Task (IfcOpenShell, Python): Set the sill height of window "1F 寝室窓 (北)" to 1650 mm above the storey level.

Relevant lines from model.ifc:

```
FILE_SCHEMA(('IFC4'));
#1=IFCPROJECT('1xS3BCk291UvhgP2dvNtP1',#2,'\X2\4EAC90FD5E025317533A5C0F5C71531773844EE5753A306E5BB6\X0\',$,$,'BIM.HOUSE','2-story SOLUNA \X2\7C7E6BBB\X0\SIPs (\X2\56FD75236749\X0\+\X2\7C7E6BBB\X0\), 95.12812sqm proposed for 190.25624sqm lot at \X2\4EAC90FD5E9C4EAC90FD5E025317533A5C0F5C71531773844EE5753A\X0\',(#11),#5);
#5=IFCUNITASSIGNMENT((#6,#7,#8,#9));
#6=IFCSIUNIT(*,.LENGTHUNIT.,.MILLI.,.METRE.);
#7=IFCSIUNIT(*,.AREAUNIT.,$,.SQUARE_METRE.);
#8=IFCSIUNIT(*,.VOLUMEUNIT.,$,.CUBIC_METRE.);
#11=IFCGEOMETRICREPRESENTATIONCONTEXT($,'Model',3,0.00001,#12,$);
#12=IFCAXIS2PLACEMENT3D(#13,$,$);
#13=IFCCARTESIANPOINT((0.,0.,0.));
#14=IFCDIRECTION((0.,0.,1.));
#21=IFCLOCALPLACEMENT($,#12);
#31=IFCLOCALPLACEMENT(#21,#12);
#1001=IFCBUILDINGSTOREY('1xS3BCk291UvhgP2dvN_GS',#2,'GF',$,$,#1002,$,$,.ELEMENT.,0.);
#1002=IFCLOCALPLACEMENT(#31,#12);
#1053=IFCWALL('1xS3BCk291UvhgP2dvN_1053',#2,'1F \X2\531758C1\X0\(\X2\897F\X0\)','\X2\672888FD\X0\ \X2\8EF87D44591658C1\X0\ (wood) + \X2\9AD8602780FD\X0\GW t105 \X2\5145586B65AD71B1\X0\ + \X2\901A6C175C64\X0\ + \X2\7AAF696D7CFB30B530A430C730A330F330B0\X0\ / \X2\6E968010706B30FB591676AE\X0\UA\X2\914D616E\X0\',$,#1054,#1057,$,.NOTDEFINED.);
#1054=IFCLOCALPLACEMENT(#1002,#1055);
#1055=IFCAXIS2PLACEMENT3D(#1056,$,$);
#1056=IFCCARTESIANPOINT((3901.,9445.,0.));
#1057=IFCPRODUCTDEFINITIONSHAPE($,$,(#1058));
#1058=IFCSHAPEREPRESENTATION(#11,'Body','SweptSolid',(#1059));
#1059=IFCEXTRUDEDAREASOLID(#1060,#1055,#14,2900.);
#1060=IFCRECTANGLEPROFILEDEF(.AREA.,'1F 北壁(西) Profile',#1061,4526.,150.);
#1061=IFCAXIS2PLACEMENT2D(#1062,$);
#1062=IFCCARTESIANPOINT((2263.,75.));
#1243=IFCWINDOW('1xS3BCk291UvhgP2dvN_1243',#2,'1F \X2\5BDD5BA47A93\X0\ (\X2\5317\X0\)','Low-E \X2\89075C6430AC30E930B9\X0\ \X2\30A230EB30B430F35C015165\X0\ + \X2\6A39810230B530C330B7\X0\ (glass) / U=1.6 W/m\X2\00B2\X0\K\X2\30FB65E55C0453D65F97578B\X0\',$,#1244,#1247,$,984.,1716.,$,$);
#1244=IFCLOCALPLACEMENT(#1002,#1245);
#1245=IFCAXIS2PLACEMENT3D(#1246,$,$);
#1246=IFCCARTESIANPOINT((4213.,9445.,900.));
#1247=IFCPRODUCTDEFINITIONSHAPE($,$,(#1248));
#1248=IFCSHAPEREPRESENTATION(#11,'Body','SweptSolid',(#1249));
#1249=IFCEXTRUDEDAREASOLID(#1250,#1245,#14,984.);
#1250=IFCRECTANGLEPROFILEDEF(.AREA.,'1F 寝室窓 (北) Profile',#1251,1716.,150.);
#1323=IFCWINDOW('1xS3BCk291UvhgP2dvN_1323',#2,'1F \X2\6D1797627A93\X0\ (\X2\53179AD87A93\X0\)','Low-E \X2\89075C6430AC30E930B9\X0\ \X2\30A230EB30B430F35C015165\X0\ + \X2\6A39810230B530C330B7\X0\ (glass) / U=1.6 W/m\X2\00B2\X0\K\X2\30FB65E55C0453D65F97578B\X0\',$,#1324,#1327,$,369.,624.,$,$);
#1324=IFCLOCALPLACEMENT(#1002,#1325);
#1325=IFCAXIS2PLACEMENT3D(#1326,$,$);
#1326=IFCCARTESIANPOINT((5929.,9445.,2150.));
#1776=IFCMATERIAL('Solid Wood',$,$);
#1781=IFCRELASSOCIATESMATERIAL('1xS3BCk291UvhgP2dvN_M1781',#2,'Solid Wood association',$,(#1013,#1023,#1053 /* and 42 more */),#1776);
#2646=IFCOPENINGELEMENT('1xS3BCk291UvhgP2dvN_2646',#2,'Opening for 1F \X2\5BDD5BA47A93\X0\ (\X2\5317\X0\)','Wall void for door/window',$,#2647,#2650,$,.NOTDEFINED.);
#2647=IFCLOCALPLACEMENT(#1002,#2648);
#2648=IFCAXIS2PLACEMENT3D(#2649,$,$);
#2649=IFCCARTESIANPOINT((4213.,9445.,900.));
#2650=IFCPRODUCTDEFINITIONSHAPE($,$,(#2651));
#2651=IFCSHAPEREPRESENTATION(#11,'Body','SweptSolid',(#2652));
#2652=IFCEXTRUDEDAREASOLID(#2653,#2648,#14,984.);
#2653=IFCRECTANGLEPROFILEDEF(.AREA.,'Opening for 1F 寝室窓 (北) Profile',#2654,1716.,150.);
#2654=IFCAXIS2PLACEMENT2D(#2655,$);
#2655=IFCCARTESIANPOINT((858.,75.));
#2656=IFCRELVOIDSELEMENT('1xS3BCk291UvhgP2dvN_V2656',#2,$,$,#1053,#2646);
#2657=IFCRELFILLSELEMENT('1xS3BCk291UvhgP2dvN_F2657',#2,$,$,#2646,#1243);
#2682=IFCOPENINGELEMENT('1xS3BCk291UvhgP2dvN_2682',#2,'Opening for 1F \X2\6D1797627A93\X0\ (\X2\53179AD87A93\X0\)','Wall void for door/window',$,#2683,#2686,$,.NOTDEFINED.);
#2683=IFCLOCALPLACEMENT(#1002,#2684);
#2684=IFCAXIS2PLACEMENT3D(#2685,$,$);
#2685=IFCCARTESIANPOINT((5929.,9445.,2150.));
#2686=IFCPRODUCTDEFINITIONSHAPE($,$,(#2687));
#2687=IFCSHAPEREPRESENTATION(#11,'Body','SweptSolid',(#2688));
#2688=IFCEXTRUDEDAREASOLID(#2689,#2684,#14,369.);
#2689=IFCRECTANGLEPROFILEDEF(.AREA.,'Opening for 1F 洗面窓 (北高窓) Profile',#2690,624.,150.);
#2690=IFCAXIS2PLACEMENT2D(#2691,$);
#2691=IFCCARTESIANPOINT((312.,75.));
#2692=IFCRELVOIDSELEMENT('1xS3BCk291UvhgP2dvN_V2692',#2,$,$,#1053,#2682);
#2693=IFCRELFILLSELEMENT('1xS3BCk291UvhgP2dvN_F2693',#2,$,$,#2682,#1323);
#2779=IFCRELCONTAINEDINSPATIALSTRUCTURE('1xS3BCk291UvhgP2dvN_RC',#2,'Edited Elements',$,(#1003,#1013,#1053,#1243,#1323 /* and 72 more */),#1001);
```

```python
import numpy as np
import ifcopenshell
import ifcopenshell.api.geometry
import ifcopenshell.geom
import ifcopenshell.util.element
import ifcopenshell.util.placement
import ifcopenshell.util.shape
import ifcopenshell.util.unit

model = ifcopenshell.open("model.ifc")
unit_scale = ifcopenshell.util.unit.calculate_unit_scale(model)

window = model.by_guid("1xS3BCk291UvhgP2dvN_1243")
opening = window.FillsVoids[0].RelatingOpeningElement
storey = ifcopenshell.util.element.get_container(window, ifc_class="IfcBuildingStorey")
level = ifcopenshell.util.placement.get_local_placement(storey.ObjectPlacement)[2, 3]

# The opening's origin need not be at the sill, so measure its lowest point.
shape = ifcopenshell.geom.create_shape(ifcopenshell.geom.settings(), opening)
bottom = ifcopenshell.util.shape.get_shape_bottom_elevation(shape, shape.geometry) / unit_scale
dz = level + 1650.0 - bottom

shift = np.array([0.0, 0.0, dz])
# The window is not placed relative to its opening, so move both.
for product in (opening, window):
    matrix = ifcopenshell.util.placement.get_local_placement(product.ObjectPlacement)
    matrix[:3, 3] += shift
    ifcopenshell.api.geometry.edit_object_placement(model, product=product, matrix=matrix, is_si=False)

print(f"moved by {dz * unit_scale:+.3f} m")

model.write("model_edited.ifc")
```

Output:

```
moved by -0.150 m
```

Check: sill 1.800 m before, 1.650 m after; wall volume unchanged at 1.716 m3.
